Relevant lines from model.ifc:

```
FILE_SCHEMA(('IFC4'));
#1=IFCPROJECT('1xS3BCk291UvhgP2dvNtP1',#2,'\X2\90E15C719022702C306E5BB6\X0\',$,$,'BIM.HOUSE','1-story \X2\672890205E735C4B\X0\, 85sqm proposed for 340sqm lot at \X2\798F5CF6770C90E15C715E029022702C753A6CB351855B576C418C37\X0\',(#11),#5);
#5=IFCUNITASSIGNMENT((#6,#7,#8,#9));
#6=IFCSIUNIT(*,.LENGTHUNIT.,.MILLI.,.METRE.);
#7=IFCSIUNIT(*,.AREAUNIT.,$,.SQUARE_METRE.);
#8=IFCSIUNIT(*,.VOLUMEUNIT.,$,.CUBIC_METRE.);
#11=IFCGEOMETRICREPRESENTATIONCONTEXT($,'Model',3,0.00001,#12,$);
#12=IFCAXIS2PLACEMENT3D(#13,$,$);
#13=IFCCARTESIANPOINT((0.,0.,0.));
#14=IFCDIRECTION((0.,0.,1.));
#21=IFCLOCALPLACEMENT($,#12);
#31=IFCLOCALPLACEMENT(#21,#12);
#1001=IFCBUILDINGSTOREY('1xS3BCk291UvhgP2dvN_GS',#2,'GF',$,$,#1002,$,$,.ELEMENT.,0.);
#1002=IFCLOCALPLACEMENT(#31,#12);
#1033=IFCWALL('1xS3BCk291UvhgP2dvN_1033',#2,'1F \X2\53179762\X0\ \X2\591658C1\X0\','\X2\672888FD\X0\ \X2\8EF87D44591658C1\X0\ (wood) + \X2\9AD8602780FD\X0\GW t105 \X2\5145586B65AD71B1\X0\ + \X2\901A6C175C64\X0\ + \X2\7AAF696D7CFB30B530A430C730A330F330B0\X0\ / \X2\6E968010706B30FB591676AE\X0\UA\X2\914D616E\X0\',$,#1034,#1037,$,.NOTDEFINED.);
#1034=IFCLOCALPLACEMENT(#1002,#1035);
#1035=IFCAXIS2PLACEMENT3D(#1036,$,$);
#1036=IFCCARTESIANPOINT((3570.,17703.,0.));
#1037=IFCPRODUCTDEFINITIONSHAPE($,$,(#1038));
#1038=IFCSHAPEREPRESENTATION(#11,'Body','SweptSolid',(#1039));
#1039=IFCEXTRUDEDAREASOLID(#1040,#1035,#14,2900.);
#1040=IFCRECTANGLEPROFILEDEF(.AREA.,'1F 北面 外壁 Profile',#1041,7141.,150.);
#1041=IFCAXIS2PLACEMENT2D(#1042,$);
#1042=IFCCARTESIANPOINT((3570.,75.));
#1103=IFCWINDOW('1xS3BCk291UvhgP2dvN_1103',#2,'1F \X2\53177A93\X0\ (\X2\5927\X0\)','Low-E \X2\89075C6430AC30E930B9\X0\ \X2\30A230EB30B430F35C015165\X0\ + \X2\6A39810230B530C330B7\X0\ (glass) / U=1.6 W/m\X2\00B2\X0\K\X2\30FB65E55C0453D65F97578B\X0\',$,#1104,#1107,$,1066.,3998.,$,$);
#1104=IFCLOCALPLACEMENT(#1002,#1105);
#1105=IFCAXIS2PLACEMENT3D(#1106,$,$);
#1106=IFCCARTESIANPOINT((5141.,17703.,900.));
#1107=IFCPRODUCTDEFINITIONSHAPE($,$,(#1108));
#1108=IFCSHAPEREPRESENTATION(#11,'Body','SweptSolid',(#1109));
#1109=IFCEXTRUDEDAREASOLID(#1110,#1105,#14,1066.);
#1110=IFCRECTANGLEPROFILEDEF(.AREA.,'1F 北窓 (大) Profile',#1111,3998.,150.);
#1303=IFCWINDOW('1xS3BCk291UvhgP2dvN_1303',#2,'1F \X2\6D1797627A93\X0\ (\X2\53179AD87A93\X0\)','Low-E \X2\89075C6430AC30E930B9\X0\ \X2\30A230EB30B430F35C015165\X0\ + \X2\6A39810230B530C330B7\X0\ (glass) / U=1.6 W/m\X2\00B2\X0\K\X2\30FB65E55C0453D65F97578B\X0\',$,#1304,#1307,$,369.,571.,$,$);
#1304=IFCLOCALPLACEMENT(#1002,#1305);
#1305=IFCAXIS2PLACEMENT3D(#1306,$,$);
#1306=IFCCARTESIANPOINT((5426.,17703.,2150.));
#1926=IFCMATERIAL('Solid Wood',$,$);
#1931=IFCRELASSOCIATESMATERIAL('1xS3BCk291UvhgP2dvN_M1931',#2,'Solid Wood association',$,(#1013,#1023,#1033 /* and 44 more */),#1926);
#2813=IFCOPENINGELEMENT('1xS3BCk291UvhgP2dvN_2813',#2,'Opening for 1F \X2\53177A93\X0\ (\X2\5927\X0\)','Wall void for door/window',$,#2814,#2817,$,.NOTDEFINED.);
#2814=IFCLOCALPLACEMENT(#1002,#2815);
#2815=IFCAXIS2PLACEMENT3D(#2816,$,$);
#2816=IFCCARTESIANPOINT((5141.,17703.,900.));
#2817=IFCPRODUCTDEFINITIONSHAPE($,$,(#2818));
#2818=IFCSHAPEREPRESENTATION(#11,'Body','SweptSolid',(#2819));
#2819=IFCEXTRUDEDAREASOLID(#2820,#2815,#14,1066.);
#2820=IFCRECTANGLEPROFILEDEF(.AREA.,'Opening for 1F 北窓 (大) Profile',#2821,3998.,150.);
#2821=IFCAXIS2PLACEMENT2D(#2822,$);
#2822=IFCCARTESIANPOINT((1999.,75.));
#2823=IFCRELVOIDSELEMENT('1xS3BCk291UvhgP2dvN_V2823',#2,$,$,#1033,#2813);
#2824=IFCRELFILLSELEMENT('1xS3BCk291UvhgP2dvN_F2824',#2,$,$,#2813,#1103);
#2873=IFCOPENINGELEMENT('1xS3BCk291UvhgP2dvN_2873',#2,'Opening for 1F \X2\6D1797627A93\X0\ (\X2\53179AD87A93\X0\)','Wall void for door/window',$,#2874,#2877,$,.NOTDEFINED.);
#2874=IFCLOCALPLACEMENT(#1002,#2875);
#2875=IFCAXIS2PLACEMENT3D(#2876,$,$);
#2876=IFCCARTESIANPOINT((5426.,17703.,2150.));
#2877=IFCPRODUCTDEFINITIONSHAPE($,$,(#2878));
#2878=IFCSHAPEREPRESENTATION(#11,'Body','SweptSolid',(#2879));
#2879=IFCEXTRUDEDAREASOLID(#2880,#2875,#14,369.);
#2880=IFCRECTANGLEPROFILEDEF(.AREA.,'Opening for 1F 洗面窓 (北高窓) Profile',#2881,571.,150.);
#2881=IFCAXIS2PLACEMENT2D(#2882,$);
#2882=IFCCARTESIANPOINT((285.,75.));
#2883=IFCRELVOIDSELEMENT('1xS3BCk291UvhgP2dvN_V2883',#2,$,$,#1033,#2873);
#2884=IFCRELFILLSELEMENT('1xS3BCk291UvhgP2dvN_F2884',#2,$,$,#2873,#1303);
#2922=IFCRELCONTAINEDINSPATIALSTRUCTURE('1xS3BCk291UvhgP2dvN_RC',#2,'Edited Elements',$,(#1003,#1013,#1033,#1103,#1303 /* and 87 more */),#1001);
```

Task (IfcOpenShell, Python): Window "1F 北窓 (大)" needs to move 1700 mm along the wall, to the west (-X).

```python
import ifcopenshell
import ifcopenshell.api.geometry
import ifcopenshell.util.placement

model = ifcopenshell.open("model.ifc")

window = model.by_guid("1xS3BCk291UvhgP2dvN_1103")
opening = window.FillsVoids[0].RelatingOpeningElement
wall = opening.VoidsElements[0].RelatingBuildingElement

wall_matrix = ifcopenshell.util.placement.get_local_placement(wall.ObjectPlacement)
shift = wall_matrix[:3, 0] * -1700.0
before = ifcopenshell.util.placement.get_local_placement(window.ObjectPlacement)[:3, 3].copy()

# The window is not placed relative to its opening, so move both.
for product in (opening, window):
    matrix = ifcopenshell.util.placement.get_local_placement(product.ObjectPlacement)
    matrix[:3, 3] += shift
    ifcopenshell.api.geometry.edit_object_placement(model, product=product, matrix=matrix, is_si=False)

after = ifcopenshell.util.placement.get_local_placement(window.ObjectPlacement)[:3, 3]
print("window moved by", (after - before).round(3) + 0.0)

model.write("model_v2.ifc")
```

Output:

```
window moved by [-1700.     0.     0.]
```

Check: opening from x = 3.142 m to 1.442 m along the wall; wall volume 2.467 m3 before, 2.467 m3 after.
